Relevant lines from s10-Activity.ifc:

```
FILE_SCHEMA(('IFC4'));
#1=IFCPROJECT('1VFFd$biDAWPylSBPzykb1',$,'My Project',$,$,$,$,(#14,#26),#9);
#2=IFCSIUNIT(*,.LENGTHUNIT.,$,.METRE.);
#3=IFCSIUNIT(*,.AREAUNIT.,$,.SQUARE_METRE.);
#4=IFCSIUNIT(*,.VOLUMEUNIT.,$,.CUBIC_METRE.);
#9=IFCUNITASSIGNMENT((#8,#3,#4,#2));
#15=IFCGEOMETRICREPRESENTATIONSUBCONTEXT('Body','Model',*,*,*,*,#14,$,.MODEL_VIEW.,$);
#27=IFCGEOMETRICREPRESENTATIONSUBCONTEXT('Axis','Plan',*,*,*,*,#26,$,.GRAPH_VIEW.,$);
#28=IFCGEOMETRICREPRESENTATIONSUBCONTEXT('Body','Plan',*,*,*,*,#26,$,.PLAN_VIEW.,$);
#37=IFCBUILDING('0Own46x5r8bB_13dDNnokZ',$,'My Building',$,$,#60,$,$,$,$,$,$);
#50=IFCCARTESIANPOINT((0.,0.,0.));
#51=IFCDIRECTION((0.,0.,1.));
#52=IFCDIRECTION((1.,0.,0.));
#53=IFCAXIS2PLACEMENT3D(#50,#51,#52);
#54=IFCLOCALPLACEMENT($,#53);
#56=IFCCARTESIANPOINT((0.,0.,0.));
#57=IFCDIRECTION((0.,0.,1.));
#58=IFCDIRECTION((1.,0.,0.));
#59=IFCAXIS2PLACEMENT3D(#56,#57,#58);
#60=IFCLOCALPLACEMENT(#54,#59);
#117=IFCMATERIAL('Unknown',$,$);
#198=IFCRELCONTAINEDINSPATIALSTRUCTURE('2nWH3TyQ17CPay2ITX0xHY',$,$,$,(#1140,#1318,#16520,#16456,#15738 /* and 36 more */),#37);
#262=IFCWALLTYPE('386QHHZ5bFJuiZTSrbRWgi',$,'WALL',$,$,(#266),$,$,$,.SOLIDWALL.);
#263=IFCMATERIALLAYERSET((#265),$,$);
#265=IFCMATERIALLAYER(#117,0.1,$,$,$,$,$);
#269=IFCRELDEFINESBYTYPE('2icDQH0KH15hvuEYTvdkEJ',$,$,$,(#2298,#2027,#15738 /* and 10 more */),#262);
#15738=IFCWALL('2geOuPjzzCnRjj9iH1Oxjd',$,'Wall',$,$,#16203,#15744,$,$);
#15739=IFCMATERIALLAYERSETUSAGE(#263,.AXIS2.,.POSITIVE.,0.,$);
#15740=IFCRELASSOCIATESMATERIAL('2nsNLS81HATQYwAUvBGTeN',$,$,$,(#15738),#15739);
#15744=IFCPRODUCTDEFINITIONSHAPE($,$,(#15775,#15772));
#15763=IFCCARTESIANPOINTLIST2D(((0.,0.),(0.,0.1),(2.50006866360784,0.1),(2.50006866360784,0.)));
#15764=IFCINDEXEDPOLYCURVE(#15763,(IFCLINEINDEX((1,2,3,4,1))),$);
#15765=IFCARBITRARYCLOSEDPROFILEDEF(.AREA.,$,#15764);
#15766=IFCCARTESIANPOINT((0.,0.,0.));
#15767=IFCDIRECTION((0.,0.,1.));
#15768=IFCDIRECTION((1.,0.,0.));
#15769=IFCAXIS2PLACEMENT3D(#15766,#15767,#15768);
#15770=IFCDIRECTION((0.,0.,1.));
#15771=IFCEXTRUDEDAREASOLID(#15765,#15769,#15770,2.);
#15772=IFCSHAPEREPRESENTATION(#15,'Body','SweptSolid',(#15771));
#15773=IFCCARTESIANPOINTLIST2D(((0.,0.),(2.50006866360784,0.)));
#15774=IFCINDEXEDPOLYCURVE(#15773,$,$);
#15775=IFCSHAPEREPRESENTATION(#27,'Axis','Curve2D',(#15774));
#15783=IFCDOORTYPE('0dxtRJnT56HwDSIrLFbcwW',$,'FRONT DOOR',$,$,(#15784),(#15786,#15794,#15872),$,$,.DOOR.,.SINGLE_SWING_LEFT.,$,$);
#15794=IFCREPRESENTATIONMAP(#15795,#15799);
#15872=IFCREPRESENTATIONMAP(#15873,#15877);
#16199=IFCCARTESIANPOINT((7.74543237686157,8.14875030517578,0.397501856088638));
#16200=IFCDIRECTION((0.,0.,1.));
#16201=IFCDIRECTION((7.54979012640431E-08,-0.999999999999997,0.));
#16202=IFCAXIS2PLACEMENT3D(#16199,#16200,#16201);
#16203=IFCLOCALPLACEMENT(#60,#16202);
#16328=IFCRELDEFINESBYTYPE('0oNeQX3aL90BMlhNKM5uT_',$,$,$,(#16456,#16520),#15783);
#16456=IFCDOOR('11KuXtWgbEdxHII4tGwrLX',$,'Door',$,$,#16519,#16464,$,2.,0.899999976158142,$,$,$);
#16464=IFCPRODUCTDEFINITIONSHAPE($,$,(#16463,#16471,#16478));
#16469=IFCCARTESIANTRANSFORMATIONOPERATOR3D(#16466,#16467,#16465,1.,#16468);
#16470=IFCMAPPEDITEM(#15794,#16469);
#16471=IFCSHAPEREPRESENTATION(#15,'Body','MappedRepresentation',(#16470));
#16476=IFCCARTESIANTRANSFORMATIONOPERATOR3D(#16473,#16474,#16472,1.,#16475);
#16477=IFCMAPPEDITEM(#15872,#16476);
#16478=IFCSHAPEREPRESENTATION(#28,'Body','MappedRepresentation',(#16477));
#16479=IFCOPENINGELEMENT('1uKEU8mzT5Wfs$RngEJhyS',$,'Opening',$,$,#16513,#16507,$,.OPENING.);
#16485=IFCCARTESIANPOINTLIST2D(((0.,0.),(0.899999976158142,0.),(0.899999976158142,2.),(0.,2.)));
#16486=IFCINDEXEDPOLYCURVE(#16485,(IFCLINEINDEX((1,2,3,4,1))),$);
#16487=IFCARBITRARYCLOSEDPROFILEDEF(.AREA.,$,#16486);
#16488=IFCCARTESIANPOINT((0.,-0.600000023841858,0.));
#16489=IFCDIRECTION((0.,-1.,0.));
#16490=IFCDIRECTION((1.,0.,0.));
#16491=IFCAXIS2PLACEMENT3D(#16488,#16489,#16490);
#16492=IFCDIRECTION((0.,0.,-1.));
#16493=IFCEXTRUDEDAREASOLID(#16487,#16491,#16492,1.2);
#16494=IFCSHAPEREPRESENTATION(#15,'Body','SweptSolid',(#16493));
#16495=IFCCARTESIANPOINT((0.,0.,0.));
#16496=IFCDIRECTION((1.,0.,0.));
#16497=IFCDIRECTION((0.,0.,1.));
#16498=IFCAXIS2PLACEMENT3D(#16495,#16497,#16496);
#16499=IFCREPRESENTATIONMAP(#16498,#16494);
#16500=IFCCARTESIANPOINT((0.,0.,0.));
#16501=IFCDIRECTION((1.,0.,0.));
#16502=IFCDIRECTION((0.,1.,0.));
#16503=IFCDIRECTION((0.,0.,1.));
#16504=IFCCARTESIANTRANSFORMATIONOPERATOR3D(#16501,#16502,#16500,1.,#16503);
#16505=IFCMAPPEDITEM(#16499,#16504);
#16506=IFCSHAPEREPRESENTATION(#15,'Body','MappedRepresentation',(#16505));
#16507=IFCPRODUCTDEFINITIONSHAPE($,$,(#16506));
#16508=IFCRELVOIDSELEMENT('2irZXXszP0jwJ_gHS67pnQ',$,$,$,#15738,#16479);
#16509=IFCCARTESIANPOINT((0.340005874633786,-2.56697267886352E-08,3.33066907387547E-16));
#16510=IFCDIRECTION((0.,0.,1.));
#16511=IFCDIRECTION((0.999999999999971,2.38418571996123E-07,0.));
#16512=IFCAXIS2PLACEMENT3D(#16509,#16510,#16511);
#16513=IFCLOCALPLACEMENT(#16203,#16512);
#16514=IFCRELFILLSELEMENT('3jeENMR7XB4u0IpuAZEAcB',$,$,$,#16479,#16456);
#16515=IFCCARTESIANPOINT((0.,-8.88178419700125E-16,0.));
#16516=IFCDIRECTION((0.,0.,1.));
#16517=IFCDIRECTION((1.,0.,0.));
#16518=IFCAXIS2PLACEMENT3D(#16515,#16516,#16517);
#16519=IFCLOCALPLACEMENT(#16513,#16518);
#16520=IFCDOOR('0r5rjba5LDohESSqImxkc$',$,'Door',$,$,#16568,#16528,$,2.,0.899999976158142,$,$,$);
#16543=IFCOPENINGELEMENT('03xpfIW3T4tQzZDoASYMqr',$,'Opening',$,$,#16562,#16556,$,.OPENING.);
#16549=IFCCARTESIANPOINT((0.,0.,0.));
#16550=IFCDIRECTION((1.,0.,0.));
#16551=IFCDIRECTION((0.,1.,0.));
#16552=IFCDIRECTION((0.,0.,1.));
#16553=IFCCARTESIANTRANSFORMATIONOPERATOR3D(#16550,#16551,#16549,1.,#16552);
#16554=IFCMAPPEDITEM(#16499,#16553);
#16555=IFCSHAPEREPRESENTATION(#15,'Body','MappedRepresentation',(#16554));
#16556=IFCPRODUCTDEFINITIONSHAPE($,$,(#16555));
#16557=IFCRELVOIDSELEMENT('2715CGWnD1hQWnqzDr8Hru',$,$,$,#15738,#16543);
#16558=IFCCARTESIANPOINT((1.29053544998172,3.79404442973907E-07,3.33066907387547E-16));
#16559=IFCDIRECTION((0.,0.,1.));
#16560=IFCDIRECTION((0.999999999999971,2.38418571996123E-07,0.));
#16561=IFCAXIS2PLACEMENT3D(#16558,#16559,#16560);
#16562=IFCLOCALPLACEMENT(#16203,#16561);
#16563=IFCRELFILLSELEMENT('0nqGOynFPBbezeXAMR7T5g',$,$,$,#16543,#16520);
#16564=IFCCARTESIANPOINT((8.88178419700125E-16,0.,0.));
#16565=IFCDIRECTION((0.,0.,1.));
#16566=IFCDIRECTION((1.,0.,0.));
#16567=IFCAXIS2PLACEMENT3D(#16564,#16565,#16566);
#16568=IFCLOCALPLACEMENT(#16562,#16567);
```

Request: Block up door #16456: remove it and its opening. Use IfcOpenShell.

```python
import ifcopenshell
import ifcopenshell.api.feature
import ifcopenshell.api.root
import ifcopenshell.geom
import ifcopenshell.util.shape

model = ifcopenshell.open("s10-Activity.ifc")
settings = ifcopenshell.geom.settings()


def volume(element):
    """Net volume in cubic metres, openings subtracted."""
    shape = ifcopenshell.geom.create_shape(settings, element)
    return ifcopenshell.util.shape.get_volume(shape.geometry)


door = model.by_guid("11KuXtWgbEdxHII4tGwrLX")
opening = door.FillsVoids[0].RelatingOpeningElement
wall = opening.VoidsElements[0].RelatingBuildingElement
before = volume(wall)

ifcopenshell.api.root.remove_product(model, product=door)
ifcopenshell.api.feature.remove_feature(model, feature=opening)

after = volume(wall)

print(f"wall volume {before:.3f} -> {after:.3f} m3")

model.write("s10-Activity_edited.ifc")
```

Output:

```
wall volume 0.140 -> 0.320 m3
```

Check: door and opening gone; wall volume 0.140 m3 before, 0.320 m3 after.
